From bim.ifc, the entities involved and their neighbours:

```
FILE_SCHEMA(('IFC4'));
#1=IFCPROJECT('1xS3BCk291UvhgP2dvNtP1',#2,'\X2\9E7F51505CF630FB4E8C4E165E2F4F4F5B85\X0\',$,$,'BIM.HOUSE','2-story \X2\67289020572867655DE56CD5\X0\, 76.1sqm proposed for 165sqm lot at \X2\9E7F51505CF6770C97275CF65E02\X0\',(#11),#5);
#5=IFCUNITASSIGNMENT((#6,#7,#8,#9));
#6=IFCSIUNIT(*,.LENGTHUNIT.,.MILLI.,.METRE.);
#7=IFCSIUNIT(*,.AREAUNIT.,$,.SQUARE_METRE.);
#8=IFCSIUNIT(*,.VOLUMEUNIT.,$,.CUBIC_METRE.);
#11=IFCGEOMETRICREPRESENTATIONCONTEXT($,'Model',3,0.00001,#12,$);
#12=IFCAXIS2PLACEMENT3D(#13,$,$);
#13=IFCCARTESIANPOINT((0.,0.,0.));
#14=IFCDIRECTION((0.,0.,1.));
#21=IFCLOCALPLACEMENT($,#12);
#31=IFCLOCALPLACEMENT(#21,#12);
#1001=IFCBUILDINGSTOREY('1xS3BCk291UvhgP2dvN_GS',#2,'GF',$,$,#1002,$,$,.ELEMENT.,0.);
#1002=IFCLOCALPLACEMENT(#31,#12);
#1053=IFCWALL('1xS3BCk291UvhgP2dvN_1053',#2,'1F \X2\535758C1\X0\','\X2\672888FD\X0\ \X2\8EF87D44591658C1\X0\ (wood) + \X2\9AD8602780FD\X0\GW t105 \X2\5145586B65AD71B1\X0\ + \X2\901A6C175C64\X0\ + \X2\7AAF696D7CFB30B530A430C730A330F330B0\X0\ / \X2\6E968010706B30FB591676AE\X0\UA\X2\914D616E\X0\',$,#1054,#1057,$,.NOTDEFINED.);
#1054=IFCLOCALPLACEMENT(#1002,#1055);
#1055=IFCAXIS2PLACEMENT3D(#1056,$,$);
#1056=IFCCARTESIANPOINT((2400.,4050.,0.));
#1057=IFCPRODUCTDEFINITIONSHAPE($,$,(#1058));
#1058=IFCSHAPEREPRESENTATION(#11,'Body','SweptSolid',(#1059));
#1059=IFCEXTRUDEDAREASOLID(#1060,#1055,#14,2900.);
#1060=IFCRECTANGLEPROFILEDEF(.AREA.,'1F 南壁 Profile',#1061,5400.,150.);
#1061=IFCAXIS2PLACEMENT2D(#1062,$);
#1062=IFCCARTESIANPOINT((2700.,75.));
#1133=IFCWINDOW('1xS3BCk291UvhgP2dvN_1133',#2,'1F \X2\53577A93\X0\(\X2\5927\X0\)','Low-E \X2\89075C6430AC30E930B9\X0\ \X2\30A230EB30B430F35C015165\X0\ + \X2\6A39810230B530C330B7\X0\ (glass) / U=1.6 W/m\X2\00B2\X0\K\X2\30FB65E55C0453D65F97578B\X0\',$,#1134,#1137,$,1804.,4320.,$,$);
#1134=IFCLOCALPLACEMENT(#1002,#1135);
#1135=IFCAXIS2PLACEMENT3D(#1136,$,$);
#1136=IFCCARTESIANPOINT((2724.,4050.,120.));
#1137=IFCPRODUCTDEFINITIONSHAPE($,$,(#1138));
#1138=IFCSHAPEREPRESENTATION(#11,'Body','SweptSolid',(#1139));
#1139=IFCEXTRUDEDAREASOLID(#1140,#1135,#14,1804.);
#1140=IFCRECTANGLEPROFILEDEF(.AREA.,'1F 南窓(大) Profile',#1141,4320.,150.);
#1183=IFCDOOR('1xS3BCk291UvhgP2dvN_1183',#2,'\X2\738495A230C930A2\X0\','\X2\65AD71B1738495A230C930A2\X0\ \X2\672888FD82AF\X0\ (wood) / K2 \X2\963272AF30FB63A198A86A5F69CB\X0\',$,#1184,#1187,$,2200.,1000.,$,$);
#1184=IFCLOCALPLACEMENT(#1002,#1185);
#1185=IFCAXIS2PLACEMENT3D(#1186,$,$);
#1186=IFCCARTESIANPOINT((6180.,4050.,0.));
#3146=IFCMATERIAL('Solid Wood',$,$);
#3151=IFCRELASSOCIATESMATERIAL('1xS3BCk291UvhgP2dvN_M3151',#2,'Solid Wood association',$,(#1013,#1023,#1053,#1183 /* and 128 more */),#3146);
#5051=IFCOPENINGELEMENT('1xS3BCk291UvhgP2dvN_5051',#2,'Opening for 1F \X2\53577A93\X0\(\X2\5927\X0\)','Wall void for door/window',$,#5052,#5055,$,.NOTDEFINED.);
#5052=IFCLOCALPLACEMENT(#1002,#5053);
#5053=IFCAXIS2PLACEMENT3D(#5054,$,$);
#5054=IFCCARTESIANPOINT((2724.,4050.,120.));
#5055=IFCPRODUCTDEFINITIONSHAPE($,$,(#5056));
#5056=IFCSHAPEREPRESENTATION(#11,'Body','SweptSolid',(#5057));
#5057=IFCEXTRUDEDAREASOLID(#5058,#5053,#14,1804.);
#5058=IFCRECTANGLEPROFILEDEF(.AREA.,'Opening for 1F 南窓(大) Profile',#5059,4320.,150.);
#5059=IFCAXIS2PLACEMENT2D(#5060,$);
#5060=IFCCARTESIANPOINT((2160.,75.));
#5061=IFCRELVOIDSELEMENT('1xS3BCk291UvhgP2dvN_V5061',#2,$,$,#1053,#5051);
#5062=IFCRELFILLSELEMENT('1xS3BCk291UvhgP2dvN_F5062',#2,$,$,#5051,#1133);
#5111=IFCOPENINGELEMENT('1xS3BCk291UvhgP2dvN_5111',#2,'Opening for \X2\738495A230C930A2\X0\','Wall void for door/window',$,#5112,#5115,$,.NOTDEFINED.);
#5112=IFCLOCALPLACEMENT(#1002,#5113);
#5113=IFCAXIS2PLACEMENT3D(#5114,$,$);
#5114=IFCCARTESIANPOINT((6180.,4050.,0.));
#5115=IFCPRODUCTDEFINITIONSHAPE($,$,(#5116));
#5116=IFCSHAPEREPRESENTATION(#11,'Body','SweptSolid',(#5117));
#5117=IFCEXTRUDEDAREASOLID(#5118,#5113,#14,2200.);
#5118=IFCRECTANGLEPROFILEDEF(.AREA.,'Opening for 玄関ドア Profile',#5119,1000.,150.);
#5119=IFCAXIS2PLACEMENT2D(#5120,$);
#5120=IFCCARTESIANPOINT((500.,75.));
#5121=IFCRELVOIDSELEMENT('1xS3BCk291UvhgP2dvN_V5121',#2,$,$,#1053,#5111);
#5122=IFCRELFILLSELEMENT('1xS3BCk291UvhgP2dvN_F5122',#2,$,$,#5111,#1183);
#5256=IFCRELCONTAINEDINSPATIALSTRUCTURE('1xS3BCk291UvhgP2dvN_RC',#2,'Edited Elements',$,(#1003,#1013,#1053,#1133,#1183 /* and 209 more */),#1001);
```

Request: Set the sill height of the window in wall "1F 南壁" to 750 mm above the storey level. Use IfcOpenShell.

```python
import numpy as np
import ifcopenshell
import ifcopenshell.api.geometry
import ifcopenshell.geom
import ifcopenshell.util.element
import ifcopenshell.util.placement
import ifcopenshell.util.shape
import ifcopenshell.util.unit

model = ifcopenshell.open("bim.ifc")
unit_scale = ifcopenshell.util.unit.calculate_unit_scale(model)

window = model.by_guid("1xS3BCk291UvhgP2dvN_1133")
opening = window.FillsVoids[0].RelatingOpeningElement
storey = ifcopenshell.util.element.get_container(window, ifc_class="IfcBuildingStorey")
level = ifcopenshell.util.placement.get_local_placement(storey.ObjectPlacement)[2, 3]

# The opening's origin need not be at the sill, so measure its lowest point.
shape = ifcopenshell.geom.create_shape(ifcopenshell.geom.settings(), opening)
bottom = ifcopenshell.util.shape.get_shape_bottom_elevation(shape, shape.geometry) / unit_scale
dz = level + 0.75 / unit_scale - bottom

shift = np.array([0.0, 0.0, dz])
# The window is not placed relative to its opening, so move both.
for product in (opening, window):
    matrix = ifcopenshell.util.placement.get_local_placement(product.ObjectPlacement)
    matrix[:3, 3] += shift
    ifcopenshell.api.geometry.edit_object_placement(model, product=product, matrix=matrix, is_si=False)

print(f"moved by {dz * unit_scale:+.3f} m")

model.write("bim_v2.ifc")
```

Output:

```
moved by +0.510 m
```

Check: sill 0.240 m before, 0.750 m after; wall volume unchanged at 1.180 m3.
